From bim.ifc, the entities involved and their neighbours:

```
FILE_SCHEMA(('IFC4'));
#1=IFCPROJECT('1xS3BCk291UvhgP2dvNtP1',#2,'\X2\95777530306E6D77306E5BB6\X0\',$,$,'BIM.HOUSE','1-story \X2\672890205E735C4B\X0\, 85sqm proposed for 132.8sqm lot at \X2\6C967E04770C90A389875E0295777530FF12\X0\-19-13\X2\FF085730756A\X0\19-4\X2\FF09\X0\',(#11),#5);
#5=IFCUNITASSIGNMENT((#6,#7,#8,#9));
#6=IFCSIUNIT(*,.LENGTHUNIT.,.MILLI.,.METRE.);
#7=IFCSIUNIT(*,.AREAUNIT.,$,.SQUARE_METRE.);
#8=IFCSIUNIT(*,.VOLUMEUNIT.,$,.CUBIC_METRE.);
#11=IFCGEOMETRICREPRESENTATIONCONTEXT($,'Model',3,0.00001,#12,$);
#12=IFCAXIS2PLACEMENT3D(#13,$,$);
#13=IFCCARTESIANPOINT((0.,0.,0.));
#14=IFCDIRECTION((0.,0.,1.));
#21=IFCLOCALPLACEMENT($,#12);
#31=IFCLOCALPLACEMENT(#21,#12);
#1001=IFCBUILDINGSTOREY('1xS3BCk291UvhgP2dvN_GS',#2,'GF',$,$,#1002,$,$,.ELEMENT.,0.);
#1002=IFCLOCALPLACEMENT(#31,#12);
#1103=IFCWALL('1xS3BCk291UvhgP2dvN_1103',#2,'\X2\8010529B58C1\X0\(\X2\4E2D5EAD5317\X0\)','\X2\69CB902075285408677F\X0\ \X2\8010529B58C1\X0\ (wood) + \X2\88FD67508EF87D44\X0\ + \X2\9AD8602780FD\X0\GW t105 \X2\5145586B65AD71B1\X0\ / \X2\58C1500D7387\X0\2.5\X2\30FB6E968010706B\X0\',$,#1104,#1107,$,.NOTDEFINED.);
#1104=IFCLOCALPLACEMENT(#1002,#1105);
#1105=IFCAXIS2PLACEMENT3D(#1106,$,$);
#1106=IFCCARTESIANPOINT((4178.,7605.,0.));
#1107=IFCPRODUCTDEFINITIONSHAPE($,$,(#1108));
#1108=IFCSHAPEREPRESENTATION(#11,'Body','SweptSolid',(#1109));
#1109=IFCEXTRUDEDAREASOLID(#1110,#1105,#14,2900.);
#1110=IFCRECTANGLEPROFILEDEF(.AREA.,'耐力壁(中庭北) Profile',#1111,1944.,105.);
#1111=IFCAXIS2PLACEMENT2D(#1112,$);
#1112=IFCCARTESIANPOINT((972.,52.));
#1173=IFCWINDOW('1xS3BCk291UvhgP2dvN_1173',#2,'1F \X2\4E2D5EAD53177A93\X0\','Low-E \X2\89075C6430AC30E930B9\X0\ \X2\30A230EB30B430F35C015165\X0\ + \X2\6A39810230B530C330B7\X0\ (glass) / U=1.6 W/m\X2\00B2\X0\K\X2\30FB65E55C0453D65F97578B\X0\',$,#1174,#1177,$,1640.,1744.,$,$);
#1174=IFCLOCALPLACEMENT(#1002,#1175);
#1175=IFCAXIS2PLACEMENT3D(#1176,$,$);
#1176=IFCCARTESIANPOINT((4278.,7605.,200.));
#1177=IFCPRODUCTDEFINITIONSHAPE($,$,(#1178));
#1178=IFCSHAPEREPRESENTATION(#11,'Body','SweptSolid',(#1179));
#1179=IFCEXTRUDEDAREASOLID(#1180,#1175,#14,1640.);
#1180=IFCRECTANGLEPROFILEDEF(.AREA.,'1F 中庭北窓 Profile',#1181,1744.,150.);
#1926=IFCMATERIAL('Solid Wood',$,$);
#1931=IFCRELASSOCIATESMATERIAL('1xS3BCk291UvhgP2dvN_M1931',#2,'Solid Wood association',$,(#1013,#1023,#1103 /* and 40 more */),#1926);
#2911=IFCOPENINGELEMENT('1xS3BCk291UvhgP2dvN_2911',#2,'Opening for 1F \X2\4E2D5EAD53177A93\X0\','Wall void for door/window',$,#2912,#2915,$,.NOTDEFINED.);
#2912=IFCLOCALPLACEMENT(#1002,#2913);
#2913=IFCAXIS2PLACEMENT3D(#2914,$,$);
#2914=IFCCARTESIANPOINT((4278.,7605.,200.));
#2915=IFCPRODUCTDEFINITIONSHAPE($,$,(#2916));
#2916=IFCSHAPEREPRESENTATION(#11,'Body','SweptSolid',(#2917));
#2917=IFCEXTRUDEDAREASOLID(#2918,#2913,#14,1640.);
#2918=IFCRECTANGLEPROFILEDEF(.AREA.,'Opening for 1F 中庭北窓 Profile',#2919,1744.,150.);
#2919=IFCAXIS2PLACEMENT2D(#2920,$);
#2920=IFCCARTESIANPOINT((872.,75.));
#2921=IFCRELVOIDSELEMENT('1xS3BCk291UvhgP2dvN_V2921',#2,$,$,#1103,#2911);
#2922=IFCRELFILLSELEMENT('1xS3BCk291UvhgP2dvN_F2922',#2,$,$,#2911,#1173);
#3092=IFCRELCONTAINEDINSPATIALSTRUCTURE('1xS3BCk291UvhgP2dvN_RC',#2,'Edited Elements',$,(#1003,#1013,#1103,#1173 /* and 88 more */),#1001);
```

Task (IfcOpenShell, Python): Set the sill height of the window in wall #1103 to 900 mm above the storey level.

```python
import numpy as np
import ifcopenshell
import ifcopenshell.api.geometry
import ifcopenshell.geom
import ifcopenshell.util.element
import ifcopenshell.util.placement
import ifcopenshell.util.shape
import ifcopenshell.util.unit

model = ifcopenshell.open("bim.ifc")
unit_scale = ifcopenshell.util.unit.calculate_unit_scale(model)

window = model.by_guid("1xS3BCk291UvhgP2dvN_1173")
opening = window.FillsVoids[0].RelatingOpeningElement
storey = ifcopenshell.util.element.get_container(window, ifc_class="IfcBuildingStorey")
level = ifcopenshell.util.placement.get_local_placement(storey.ObjectPlacement)[2, 3]

# The opening's origin need not be at the sill, so measure its lowest point.
shape = ifcopenshell.geom.create_shape(ifcopenshell.geom.settings(), opening)
bottom = ifcopenshell.util.shape.get_shape_bottom_elevation(shape, shape.geometry) / unit_scale
dz = level + 0.9 / unit_scale - bottom

shift = np.array([0.0, 0.0, dz])
# The window is not placed relative to its opening, so move both.
for product in (opening, window):
    matrix = ifcopenshell.util.placement.get_local_placement(product.ObjectPlacement)
    matrix[:3, 3] += shift
    ifcopenshell.api.geometry.edit_object_placement(model, product=product, matrix=matrix, is_si=False)

print(f"moved by {dz * unit_scale:+.3f} m")

model.write("bim-out.ifc")
```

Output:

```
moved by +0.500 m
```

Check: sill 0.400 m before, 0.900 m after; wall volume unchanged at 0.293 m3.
